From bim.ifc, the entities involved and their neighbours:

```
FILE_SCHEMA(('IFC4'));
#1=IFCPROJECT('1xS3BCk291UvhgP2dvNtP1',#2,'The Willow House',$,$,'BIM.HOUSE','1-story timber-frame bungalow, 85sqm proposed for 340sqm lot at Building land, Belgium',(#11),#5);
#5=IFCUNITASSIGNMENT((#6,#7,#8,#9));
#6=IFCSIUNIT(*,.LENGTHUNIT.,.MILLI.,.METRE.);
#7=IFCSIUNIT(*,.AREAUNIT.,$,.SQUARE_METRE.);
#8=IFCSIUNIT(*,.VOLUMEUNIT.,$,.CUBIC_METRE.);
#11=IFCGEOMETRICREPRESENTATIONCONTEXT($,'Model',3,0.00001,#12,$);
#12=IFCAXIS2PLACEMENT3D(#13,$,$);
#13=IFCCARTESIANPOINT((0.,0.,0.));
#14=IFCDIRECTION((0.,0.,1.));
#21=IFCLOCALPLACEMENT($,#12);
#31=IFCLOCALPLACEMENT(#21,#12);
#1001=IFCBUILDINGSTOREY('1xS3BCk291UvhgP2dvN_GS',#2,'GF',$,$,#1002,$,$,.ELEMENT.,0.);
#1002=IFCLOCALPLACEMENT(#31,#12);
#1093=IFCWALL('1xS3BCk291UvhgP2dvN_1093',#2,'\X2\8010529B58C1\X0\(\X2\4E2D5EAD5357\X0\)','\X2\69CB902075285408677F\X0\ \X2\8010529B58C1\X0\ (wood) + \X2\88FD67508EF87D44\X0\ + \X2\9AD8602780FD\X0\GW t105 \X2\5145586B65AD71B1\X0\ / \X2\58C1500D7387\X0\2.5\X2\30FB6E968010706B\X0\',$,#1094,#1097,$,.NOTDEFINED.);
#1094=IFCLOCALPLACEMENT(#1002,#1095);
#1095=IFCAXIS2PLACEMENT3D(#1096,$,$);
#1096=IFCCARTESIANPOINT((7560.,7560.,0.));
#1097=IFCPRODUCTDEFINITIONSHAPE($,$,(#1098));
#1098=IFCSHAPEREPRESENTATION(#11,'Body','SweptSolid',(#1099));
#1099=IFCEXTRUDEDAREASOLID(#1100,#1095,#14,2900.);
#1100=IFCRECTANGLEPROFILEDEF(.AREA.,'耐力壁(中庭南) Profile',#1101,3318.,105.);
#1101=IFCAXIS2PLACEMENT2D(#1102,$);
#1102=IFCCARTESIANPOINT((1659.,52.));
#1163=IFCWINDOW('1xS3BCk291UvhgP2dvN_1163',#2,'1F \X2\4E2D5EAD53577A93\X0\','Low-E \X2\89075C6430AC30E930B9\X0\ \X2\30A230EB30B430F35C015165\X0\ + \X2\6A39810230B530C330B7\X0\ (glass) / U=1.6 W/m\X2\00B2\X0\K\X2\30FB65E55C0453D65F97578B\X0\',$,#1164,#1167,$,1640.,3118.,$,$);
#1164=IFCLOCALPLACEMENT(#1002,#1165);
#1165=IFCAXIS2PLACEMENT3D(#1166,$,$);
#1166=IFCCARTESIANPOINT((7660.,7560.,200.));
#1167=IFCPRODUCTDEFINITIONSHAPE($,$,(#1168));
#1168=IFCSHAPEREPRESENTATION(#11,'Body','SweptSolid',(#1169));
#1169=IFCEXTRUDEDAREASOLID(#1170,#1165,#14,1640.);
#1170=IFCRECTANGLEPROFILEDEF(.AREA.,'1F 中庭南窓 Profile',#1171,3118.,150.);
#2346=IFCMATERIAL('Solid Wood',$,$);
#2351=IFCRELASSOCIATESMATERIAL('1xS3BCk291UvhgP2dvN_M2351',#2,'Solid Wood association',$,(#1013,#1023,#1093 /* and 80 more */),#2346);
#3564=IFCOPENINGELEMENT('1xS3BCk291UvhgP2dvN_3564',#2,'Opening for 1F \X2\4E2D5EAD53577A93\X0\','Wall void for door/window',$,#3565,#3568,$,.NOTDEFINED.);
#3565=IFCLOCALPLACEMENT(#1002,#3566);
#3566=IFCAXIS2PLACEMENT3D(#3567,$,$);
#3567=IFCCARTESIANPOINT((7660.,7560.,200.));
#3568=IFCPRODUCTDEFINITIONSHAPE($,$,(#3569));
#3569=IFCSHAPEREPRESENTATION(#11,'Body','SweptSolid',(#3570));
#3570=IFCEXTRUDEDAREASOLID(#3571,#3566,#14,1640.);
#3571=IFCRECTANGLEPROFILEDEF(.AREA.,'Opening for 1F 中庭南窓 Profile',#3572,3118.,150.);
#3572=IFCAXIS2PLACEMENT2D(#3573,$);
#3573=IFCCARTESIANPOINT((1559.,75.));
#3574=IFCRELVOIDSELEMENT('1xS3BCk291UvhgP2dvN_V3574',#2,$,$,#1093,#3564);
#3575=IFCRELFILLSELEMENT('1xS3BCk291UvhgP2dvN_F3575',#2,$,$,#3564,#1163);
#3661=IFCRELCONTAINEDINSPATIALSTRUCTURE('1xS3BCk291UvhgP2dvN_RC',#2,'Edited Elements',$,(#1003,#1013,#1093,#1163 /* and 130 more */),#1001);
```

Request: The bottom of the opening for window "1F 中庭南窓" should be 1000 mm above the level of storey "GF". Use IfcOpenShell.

```python
import numpy as np
import ifcopenshell
import ifcopenshell.api.geometry
import ifcopenshell.geom
import ifcopenshell.util.element
import ifcopenshell.util.placement
import ifcopenshell.util.shape
import ifcopenshell.util.unit

model = ifcopenshell.open("bim.ifc")
unit_scale = ifcopenshell.util.unit.calculate_unit_scale(model)

window = model.by_guid("1xS3BCk291UvhgP2dvN_1163")
opening = window.FillsVoids[0].RelatingOpeningElement
storey = ifcopenshell.util.element.get_container(window, ifc_class="IfcBuildingStorey")
level = ifcopenshell.util.placement.get_local_placement(storey.ObjectPlacement)[2, 3]

# The opening's origin need not be at the sill, so measure its lowest point.
shape = ifcopenshell.geom.create_shape(ifcopenshell.geom.settings(), opening)
bottom = ifcopenshell.util.shape.get_shape_bottom_elevation(shape, shape.geometry) / unit_scale
dz = level + 1 / unit_scale - bottom

shift = np.array([0.0, 0.0, dz])
# The window is not placed relative to its opening, so move both.
for product in (opening, window):
    matrix = ifcopenshell.util.placement.get_local_placement(product.ObjectPlacement)
    matrix[:3, 3] += shift
    ifcopenshell.api.geometry.edit_object_placement(model, product=product, matrix=matrix, is_si=False)

print(f"moved by {dz * unit_scale:+.3f} m")

model.write("bim_edited.ifc")
```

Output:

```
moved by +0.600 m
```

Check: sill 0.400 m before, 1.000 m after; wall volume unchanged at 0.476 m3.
